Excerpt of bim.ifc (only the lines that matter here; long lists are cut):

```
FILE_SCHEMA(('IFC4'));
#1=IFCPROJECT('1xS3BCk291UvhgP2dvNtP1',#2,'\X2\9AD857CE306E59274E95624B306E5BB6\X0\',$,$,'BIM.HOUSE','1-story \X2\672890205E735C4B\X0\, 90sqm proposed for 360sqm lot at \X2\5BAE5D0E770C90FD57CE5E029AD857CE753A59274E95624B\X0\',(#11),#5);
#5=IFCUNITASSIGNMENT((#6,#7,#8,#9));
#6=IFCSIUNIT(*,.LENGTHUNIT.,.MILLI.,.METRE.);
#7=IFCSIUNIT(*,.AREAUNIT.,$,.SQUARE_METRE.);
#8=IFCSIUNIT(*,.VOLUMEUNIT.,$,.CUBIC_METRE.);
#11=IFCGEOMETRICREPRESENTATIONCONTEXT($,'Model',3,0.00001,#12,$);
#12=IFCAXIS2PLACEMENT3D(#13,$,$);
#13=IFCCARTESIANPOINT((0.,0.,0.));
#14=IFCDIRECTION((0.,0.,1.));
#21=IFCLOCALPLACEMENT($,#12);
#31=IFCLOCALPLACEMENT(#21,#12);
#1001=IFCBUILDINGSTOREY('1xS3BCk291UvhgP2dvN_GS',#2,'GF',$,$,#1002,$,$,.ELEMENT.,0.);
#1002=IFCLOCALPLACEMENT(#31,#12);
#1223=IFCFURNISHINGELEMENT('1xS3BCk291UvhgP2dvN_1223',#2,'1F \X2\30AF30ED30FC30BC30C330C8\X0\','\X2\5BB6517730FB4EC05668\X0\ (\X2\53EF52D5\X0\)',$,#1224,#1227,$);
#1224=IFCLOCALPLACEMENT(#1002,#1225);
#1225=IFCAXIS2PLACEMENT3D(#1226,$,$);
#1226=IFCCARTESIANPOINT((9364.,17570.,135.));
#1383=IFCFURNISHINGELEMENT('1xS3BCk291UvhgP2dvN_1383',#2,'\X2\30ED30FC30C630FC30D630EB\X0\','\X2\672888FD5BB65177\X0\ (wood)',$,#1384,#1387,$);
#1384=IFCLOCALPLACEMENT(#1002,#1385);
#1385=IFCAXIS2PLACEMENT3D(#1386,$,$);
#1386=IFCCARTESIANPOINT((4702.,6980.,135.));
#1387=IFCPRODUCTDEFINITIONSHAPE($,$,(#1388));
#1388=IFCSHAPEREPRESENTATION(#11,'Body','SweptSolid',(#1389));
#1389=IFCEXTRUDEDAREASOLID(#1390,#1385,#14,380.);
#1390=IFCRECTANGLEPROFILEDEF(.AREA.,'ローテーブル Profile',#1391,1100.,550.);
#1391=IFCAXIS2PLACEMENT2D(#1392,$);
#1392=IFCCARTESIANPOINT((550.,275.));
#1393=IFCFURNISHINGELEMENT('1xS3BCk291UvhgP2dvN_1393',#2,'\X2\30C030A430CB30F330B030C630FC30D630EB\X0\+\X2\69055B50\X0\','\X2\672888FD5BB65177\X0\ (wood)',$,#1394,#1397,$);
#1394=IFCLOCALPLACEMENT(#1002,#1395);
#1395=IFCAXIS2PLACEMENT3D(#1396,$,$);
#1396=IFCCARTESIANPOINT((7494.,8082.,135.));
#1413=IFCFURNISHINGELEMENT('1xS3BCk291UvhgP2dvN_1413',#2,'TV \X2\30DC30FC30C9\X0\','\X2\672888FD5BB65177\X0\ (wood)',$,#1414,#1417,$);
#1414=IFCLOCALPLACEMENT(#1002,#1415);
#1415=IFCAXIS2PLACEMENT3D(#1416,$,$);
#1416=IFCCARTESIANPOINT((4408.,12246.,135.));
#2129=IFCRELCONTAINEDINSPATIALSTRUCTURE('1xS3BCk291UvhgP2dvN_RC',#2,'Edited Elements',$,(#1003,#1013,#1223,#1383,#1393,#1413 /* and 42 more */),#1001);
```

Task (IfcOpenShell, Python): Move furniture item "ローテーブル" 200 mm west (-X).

```python
import ifcopenshell
import ifcopenshell.api.geometry
import ifcopenshell.util.placement

model = ifcopenshell.open("bim.ifc")

item = model.by_guid("1xS3BCk291UvhgP2dvN_1383")
matrix = ifcopenshell.util.placement.get_local_placement(item.ObjectPlacement)
matrix[0, 3] -= 200.0
ifcopenshell.api.geometry.edit_object_placement(model, product=item, matrix=matrix, is_si=False)

print(ifcopenshell.util.placement.get_local_placement(item.ObjectPlacement).round(3) + 0.0)

model.write("bim_updated.ifc")
```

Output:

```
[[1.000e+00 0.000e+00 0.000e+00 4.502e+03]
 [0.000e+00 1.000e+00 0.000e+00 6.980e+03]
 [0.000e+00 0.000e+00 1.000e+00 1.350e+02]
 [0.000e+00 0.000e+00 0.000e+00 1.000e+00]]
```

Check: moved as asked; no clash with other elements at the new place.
